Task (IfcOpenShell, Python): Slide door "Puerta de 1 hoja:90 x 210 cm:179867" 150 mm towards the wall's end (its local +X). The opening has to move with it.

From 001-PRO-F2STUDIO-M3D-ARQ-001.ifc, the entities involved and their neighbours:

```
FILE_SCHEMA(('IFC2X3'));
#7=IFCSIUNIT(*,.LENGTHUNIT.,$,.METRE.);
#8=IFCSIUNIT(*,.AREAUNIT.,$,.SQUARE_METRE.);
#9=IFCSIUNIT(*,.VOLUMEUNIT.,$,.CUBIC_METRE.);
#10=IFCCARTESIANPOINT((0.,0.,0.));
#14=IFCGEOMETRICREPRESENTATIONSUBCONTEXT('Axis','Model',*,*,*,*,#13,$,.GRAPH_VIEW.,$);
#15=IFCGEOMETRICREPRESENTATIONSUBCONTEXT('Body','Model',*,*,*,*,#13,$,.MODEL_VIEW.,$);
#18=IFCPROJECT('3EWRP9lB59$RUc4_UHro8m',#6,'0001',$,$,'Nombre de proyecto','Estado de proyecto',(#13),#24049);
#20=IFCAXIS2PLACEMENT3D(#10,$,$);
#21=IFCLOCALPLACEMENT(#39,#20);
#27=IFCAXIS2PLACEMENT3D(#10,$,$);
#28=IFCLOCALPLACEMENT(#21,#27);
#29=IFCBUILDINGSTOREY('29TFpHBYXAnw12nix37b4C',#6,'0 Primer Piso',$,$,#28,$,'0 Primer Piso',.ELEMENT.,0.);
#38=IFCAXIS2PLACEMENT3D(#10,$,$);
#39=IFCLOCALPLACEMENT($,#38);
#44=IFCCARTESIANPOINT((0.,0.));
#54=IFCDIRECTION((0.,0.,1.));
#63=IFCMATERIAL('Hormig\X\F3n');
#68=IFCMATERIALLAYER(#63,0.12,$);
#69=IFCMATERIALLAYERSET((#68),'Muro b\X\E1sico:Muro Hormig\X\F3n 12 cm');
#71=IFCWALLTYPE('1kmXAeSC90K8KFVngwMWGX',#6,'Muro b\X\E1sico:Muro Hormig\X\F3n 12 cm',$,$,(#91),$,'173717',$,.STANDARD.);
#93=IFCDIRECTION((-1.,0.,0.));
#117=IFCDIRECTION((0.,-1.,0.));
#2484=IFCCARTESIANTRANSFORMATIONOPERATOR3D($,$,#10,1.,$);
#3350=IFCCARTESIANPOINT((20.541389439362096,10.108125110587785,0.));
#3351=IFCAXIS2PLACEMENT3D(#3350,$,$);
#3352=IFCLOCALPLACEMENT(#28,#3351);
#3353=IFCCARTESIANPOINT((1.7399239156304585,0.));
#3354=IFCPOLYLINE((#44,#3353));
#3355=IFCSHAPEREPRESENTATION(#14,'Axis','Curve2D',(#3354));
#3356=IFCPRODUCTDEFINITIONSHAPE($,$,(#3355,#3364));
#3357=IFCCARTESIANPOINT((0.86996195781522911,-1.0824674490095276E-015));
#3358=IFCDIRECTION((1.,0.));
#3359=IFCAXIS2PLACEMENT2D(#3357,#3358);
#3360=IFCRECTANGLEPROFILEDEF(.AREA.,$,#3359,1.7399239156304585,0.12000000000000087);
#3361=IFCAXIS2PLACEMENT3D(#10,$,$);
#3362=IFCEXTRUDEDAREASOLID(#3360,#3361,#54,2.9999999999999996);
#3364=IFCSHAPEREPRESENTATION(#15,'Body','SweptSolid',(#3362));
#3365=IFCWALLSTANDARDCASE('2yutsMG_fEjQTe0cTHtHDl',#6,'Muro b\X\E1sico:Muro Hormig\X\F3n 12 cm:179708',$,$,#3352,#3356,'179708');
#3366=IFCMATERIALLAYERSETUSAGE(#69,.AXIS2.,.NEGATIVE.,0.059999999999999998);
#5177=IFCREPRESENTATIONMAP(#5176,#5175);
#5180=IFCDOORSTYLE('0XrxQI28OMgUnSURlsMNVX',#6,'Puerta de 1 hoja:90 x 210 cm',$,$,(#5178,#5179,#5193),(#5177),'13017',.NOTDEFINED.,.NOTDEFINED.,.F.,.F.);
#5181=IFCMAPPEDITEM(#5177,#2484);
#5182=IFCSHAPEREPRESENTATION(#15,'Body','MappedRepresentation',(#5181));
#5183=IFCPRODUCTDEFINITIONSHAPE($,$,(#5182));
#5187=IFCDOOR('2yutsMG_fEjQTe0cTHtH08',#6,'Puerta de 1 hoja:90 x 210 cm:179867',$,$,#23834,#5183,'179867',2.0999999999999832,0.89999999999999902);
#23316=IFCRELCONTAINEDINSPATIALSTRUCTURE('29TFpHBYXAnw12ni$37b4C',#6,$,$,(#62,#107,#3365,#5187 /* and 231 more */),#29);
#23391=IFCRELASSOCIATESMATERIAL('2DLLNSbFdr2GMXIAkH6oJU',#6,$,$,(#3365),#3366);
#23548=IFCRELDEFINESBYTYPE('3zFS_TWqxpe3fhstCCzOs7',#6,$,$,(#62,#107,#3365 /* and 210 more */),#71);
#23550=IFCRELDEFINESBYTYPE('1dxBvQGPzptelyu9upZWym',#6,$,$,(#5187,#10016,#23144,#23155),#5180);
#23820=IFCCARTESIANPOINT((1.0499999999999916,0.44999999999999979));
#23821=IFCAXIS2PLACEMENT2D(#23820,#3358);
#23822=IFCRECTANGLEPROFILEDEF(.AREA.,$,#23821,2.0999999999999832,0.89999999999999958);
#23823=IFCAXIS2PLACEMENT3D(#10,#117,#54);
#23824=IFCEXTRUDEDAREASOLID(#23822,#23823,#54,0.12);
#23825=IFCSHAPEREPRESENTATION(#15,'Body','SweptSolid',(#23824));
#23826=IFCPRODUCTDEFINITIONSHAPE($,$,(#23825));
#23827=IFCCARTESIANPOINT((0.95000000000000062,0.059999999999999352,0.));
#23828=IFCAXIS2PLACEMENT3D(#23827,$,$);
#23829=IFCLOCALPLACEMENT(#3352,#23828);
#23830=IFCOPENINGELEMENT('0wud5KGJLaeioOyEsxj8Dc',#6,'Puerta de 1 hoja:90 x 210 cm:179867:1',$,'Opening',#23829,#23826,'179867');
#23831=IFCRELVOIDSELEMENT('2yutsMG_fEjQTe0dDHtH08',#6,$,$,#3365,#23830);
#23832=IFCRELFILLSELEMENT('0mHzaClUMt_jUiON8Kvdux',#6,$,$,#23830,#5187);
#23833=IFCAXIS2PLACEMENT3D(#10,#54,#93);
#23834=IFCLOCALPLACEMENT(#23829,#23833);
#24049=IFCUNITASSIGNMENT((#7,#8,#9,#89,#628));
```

```python
import ifcopenshell
import ifcopenshell.api.geometry
import ifcopenshell.util.placement
import ifcopenshell.util.unit

model = ifcopenshell.open("001-PRO-F2STUDIO-M3D-ARQ-001.ifc")
unit_scale = ifcopenshell.util.unit.calculate_unit_scale(model)

door = model.by_guid("2yutsMG_fEjQTe0cTHtH08")
opening = door.FillsVoids[0].RelatingOpeningElement
wall = opening.VoidsElements[0].RelatingBuildingElement

wall_matrix = ifcopenshell.util.placement.get_local_placement(wall.ObjectPlacement)
shift = wall_matrix[:3, 0] * 0.15 / unit_scale
before = ifcopenshell.util.placement.get_local_placement(door.ObjectPlacement)[:3, 3].copy()

# The door is placed relative to its opening, so it follows when the opening moves.
matrix = ifcopenshell.util.placement.get_local_placement(opening.ObjectPlacement)
matrix[:3, 3] += shift
ifcopenshell.api.geometry.edit_object_placement(
    model, product=opening, matrix=matrix, is_si=False, should_transform_children=True
)

after = ifcopenshell.util.placement.get_local_placement(door.ObjectPlacement)[:3, 3]
print("door moved by", (after - before).round(3) + 0.0)

model.write("001-PRO-F2STUDIO-M3D-ARQ-001_updated.ifc")
```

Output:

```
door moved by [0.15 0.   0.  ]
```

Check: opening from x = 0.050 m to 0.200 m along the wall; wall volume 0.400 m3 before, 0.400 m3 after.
